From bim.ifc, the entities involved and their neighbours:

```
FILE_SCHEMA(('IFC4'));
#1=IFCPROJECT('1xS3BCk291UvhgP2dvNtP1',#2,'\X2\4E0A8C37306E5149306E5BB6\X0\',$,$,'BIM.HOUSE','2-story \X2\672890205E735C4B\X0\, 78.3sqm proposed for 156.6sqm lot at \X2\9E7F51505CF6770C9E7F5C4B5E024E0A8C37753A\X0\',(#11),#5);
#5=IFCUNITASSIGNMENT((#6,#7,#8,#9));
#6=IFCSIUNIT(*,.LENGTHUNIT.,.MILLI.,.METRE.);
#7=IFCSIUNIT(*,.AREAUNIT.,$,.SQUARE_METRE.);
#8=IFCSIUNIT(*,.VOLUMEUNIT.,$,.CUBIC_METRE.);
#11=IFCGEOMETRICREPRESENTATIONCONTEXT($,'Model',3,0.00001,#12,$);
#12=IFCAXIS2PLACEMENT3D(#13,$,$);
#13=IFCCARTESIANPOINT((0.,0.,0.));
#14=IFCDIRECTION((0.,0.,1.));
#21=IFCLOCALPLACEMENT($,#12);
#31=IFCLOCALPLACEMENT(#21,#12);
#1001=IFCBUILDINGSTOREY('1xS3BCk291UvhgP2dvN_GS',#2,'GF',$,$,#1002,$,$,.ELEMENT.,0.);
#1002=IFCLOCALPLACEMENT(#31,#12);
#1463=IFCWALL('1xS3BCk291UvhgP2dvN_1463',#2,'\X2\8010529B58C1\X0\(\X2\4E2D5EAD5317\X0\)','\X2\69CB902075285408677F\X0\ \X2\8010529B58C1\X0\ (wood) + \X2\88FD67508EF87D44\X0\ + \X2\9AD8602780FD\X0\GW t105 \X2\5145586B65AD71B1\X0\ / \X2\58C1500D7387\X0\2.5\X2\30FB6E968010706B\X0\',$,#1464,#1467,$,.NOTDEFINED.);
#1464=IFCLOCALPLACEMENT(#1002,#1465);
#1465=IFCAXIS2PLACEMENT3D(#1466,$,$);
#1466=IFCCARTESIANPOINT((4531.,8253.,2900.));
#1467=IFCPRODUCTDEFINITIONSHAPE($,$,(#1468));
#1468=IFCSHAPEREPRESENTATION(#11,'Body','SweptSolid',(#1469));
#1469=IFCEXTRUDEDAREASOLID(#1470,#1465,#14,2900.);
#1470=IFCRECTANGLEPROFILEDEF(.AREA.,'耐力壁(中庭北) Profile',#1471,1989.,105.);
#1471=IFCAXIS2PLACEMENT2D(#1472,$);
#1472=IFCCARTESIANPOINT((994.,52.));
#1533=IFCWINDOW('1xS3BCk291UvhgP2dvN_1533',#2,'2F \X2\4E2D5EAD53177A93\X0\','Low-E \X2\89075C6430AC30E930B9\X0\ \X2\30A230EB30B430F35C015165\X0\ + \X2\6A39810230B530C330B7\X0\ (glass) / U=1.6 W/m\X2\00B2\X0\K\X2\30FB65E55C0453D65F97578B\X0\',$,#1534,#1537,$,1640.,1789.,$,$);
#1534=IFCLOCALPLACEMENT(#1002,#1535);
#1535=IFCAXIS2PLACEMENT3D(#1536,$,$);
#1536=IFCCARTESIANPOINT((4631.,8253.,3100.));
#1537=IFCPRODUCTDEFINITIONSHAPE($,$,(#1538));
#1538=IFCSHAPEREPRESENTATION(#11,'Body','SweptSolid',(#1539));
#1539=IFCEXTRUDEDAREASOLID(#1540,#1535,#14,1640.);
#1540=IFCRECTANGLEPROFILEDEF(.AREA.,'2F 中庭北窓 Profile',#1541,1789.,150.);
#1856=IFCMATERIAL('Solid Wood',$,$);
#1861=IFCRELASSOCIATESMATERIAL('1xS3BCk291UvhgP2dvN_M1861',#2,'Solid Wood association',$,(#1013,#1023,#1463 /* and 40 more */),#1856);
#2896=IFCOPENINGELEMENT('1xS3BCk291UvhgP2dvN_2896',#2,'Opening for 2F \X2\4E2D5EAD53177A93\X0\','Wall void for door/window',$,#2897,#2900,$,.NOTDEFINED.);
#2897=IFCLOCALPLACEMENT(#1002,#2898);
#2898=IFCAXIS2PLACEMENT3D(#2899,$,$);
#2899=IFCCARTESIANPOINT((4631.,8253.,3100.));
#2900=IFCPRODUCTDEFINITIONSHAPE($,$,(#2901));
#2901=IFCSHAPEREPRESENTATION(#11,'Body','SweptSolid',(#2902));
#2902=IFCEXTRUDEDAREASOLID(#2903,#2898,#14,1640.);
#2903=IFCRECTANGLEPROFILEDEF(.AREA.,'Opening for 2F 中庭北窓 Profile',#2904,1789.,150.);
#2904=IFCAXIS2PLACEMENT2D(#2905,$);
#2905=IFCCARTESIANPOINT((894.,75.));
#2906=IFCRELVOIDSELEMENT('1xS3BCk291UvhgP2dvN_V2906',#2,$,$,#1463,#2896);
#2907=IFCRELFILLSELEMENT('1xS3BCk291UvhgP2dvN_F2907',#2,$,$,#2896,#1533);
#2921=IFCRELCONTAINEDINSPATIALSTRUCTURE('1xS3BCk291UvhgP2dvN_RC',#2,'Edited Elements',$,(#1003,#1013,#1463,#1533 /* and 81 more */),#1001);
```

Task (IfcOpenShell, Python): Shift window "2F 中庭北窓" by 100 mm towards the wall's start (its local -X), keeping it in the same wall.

```python
import ifcopenshell
import ifcopenshell.api.geometry
import ifcopenshell.util.placement

model = ifcopenshell.open("bim.ifc")

window = model.by_guid("1xS3BCk291UvhgP2dvN_1533")
opening = window.FillsVoids[0].RelatingOpeningElement
wall = opening.VoidsElements[0].RelatingBuildingElement

wall_matrix = ifcopenshell.util.placement.get_local_placement(wall.ObjectPlacement)
shift = wall_matrix[:3, 0] * -100.0
before = ifcopenshell.util.placement.get_local_placement(window.ObjectPlacement)[:3, 3].copy()

# The window is not placed relative to its opening, so move both.
for product in (opening, window):
    matrix = ifcopenshell.util.placement.get_local_placement(product.ObjectPlacement)
    matrix[:3, 3] += shift
    ifcopenshell.api.geometry.edit_object_placement(model, product=product, matrix=matrix, is_si=False)

after = ifcopenshell.util.placement.get_local_placement(window.ObjectPlacement)[:3, 3]
print("window moved by", (after - before).round(3) + 0.0)

model.write("bim_edited.ifc")
```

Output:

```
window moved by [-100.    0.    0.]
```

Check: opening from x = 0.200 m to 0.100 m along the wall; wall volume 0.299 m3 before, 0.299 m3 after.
